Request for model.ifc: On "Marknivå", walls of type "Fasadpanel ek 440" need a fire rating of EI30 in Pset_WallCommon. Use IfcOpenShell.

First a look at what the model holds.

```python
import ifcopenshell
import ifcopenshell.util.element

model = ifcopenshell.open("model.ifc")
print(model.schema)
storey = next(s for s in model.by_type("IfcBuildingStorey") if s.Name == "Marknivå")
walls = [e for e in ifcopenshell.util.element.get_decomposition(storey) if e.is_a("IfcWall")]
seen = {}
for e in walls:
    element_type = ifcopenshell.util.element.get_type(e)
    key = (element_type.Name if element_type != e and element_type else None, ifcopenshell.util.element.get_pset(e, "Pset_WallCommon", "FireRating"))
    seen[key] = seen.get(key, 0) + 1
for (name, value), count in sorted(seen.items(), key=str):
    print(count, "x", name, "|", value)
```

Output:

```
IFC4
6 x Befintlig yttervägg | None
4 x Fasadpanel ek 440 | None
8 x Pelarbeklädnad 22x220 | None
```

```python
import ifcopenshell
import ifcopenshell.api.pset
import ifcopenshell.util.element

model = ifcopenshell.open("model.ifc")

storey = next(s for s in model.by_type("IfcBuildingStorey") if s.Name == "Marknivå")
walls = [e for e in ifcopenshell.util.element.get_decomposition(storey) if e.is_a("IfcWall")]

count = 0
for e in walls:
    element_type = ifcopenshell.util.element.get_type(e)
    if element_type in (None, e) or element_type.Name != "Fasadpanel ek 440":
        continue
    # add_pset returns the element's existing set when there is one.
    pset = ifcopenshell.api.pset.add_pset(model, product=e, name="Pset_WallCommon")
    ifcopenshell.api.pset.edit_pset(model, pset=pset, properties={"FireRating": "EI30"})
    count += 1

print(count, "walls updated")

model.write("model_v2.ifc")
```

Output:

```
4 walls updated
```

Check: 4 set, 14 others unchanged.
